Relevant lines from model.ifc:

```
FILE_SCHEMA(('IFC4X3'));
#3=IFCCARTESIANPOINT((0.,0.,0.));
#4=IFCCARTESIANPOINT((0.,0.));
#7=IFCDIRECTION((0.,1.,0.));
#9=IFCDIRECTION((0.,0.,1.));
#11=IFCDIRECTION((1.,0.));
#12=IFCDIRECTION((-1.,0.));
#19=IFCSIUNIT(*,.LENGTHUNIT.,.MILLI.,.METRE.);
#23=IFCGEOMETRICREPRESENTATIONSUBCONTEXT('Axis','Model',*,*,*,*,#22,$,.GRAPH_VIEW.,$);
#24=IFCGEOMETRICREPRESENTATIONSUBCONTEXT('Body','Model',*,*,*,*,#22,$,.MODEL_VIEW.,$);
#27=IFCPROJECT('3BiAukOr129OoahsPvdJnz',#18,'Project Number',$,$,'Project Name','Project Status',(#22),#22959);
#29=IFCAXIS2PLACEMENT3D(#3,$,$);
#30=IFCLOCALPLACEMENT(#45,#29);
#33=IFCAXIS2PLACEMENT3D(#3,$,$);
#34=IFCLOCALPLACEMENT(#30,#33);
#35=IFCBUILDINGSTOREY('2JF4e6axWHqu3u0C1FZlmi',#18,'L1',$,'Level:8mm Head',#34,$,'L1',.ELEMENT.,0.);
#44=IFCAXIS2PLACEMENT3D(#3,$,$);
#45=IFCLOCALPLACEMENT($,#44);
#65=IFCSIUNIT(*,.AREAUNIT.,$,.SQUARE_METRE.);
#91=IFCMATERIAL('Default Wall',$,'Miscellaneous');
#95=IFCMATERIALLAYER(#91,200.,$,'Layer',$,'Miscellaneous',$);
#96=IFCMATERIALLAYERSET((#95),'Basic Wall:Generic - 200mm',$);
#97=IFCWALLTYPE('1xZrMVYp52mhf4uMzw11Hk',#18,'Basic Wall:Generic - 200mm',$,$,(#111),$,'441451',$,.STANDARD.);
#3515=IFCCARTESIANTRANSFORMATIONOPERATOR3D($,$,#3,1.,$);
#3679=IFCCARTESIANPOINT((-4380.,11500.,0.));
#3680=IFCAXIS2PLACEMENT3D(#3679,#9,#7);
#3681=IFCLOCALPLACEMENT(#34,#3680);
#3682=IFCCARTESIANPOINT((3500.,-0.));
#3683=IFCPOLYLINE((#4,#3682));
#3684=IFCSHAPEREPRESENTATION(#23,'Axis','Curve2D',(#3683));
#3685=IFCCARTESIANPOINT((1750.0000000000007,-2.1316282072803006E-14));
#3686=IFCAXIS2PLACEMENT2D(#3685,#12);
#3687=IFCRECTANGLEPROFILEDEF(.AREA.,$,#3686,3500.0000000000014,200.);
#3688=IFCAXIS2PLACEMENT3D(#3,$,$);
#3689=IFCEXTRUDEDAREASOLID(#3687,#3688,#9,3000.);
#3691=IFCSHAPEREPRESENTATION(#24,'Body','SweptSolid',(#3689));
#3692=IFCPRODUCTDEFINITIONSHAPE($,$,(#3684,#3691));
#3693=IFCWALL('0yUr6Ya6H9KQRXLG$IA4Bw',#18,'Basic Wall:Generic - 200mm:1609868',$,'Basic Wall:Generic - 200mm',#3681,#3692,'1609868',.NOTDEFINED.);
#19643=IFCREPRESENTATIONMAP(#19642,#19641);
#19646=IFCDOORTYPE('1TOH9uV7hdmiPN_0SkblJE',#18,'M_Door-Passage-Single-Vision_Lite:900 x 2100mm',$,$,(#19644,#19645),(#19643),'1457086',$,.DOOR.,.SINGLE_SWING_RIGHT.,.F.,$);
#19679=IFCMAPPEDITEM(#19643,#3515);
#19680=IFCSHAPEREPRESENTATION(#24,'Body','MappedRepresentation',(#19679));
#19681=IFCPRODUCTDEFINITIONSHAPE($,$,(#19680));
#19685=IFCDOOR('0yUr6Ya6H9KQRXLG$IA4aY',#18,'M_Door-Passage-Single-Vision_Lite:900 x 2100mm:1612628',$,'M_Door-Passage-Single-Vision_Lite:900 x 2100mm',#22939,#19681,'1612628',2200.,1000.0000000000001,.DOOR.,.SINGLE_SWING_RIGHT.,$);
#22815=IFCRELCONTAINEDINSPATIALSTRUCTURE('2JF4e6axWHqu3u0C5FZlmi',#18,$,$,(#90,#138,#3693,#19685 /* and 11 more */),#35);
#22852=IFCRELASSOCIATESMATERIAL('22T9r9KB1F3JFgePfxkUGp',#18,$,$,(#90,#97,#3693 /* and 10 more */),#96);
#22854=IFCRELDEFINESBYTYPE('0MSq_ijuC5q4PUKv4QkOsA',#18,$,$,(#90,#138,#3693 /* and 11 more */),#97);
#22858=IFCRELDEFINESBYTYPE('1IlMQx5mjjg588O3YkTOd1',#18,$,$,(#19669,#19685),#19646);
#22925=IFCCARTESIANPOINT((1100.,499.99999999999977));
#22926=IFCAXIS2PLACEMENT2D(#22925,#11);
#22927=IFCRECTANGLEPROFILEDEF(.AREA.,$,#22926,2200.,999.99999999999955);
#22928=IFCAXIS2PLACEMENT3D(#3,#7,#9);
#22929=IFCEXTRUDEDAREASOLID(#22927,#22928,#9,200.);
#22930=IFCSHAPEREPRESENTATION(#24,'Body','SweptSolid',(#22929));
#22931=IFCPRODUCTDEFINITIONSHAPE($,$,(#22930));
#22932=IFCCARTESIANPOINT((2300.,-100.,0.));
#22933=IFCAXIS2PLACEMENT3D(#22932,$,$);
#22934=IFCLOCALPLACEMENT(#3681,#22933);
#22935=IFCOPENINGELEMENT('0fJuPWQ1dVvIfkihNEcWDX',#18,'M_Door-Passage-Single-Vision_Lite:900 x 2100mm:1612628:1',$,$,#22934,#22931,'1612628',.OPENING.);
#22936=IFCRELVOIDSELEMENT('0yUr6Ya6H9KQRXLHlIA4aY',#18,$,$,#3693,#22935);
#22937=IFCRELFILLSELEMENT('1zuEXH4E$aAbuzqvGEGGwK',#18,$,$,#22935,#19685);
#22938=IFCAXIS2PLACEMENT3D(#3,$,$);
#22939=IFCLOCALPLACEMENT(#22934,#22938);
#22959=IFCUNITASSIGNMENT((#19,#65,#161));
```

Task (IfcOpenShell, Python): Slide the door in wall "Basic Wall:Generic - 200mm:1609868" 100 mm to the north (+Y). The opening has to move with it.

```python
import ifcopenshell
import ifcopenshell.api.geometry
import ifcopenshell.util.placement

model = ifcopenshell.open("model.ifc")

door = model.by_id(19685)
opening = door.FillsVoids[0].RelatingOpeningElement
wall = opening.VoidsElements[0].RelatingBuildingElement

wall_matrix = ifcopenshell.util.placement.get_local_placement(wall.ObjectPlacement)
shift = wall_matrix[:3, 0] * 100.0
before = ifcopenshell.util.placement.get_local_placement(door.ObjectPlacement)[:3, 3].copy()

# The door is placed relative to its opening, so it follows when the opening moves.
matrix = ifcopenshell.util.placement.get_local_placement(opening.ObjectPlacement)
matrix[:3, 3] += shift
ifcopenshell.api.geometry.edit_object_placement(
    model, product=opening, matrix=matrix, is_si=False, should_transform_children=True
)

after = ifcopenshell.util.placement.get_local_placement(door.ObjectPlacement)[:3, 3]
print("door moved by", (after - before).round(3) + 0.0)

model.write("model_v2.ifc")
```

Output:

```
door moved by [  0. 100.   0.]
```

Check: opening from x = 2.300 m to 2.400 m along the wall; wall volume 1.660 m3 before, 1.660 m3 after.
